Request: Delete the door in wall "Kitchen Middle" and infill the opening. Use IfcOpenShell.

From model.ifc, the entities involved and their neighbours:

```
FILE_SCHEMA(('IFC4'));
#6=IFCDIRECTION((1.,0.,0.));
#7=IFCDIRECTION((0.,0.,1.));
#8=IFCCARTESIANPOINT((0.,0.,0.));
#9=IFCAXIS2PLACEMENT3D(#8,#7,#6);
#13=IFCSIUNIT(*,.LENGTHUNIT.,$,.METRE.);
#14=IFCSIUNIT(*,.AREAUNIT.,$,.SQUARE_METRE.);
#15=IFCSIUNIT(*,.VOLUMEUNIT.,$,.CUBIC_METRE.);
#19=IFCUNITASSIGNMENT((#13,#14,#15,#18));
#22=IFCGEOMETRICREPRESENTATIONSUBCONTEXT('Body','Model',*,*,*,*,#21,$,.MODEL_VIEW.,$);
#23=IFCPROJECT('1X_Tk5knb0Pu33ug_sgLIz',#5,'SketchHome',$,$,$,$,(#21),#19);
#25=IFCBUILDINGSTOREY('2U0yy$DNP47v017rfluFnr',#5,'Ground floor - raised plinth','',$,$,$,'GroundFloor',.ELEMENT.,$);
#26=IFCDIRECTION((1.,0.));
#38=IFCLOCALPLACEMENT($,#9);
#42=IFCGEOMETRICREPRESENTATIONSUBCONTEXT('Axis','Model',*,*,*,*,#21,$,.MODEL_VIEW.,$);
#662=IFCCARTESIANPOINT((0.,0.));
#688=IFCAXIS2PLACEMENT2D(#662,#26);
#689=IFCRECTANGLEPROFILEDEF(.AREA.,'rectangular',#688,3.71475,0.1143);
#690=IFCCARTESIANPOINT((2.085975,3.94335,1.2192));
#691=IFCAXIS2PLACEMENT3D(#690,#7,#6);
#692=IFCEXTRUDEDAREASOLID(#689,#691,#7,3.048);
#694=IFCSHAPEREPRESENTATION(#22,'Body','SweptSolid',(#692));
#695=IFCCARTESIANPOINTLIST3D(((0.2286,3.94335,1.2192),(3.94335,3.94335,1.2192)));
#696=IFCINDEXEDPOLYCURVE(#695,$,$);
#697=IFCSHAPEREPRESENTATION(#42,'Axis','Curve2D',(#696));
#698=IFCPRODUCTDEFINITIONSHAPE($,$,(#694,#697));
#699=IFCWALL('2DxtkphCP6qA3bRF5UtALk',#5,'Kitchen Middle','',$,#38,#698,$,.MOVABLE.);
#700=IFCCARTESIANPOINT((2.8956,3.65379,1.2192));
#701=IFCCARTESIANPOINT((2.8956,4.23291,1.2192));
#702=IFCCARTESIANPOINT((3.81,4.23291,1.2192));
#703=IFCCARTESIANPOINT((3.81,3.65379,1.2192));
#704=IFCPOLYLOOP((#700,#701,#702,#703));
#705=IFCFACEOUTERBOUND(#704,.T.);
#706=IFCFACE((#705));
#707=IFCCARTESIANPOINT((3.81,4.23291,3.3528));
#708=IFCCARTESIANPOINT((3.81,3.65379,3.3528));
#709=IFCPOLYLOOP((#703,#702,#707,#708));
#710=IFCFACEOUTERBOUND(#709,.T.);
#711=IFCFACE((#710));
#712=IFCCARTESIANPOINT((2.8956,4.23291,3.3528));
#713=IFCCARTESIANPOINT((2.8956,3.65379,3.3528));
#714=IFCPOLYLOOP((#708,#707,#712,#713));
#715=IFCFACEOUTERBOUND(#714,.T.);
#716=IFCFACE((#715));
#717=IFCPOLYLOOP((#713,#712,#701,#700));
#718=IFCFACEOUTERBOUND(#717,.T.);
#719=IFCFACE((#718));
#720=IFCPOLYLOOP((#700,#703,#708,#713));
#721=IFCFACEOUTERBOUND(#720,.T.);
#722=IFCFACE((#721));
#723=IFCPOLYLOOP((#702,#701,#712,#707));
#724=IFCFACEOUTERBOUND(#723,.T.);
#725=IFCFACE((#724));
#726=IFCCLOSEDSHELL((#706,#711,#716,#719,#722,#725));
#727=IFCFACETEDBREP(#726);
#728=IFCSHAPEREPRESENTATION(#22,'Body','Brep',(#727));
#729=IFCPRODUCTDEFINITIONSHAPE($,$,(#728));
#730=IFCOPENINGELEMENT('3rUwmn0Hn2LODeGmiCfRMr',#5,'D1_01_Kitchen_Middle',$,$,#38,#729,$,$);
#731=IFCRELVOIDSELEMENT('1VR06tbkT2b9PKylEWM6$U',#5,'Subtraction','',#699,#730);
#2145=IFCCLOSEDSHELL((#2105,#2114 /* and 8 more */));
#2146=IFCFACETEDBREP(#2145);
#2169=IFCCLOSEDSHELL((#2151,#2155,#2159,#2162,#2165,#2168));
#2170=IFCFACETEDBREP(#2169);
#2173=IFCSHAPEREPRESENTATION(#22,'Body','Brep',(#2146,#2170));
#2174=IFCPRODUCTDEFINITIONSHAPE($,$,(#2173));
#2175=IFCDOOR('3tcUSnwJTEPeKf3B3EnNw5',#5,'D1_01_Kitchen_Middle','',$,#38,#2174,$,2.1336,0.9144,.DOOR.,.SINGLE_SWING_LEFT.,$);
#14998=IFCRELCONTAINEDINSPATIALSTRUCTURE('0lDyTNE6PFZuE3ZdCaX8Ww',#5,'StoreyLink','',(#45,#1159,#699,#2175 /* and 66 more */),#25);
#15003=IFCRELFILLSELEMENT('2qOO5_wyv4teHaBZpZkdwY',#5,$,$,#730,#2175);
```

```python
import ifcopenshell
import ifcopenshell.api.feature
import ifcopenshell.api.root
import ifcopenshell.geom
import ifcopenshell.util.shape

model = ifcopenshell.open("model.ifc")
settings = ifcopenshell.geom.settings()


def volume(element):
    """Net volume in cubic metres, openings subtracted."""
    shape = ifcopenshell.geom.create_shape(settings, element)
    return ifcopenshell.util.shape.get_volume(shape.geometry)


door = model.by_guid("3tcUSnwJTEPeKf3B3EnNw5")
opening = door.FillsVoids[0].RelatingOpeningElement
wall = opening.VoidsElements[0].RelatingBuildingElement
before = volume(wall)

ifcopenshell.api.root.remove_product(model, product=door)
ifcopenshell.api.feature.remove_feature(model, feature=opening)

after = volume(wall)

print(f"wall volume {before:.3f} -> {after:.3f} m3")

model.write("model_v2.ifc")
```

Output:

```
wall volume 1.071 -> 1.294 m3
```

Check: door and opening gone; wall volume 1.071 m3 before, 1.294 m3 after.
